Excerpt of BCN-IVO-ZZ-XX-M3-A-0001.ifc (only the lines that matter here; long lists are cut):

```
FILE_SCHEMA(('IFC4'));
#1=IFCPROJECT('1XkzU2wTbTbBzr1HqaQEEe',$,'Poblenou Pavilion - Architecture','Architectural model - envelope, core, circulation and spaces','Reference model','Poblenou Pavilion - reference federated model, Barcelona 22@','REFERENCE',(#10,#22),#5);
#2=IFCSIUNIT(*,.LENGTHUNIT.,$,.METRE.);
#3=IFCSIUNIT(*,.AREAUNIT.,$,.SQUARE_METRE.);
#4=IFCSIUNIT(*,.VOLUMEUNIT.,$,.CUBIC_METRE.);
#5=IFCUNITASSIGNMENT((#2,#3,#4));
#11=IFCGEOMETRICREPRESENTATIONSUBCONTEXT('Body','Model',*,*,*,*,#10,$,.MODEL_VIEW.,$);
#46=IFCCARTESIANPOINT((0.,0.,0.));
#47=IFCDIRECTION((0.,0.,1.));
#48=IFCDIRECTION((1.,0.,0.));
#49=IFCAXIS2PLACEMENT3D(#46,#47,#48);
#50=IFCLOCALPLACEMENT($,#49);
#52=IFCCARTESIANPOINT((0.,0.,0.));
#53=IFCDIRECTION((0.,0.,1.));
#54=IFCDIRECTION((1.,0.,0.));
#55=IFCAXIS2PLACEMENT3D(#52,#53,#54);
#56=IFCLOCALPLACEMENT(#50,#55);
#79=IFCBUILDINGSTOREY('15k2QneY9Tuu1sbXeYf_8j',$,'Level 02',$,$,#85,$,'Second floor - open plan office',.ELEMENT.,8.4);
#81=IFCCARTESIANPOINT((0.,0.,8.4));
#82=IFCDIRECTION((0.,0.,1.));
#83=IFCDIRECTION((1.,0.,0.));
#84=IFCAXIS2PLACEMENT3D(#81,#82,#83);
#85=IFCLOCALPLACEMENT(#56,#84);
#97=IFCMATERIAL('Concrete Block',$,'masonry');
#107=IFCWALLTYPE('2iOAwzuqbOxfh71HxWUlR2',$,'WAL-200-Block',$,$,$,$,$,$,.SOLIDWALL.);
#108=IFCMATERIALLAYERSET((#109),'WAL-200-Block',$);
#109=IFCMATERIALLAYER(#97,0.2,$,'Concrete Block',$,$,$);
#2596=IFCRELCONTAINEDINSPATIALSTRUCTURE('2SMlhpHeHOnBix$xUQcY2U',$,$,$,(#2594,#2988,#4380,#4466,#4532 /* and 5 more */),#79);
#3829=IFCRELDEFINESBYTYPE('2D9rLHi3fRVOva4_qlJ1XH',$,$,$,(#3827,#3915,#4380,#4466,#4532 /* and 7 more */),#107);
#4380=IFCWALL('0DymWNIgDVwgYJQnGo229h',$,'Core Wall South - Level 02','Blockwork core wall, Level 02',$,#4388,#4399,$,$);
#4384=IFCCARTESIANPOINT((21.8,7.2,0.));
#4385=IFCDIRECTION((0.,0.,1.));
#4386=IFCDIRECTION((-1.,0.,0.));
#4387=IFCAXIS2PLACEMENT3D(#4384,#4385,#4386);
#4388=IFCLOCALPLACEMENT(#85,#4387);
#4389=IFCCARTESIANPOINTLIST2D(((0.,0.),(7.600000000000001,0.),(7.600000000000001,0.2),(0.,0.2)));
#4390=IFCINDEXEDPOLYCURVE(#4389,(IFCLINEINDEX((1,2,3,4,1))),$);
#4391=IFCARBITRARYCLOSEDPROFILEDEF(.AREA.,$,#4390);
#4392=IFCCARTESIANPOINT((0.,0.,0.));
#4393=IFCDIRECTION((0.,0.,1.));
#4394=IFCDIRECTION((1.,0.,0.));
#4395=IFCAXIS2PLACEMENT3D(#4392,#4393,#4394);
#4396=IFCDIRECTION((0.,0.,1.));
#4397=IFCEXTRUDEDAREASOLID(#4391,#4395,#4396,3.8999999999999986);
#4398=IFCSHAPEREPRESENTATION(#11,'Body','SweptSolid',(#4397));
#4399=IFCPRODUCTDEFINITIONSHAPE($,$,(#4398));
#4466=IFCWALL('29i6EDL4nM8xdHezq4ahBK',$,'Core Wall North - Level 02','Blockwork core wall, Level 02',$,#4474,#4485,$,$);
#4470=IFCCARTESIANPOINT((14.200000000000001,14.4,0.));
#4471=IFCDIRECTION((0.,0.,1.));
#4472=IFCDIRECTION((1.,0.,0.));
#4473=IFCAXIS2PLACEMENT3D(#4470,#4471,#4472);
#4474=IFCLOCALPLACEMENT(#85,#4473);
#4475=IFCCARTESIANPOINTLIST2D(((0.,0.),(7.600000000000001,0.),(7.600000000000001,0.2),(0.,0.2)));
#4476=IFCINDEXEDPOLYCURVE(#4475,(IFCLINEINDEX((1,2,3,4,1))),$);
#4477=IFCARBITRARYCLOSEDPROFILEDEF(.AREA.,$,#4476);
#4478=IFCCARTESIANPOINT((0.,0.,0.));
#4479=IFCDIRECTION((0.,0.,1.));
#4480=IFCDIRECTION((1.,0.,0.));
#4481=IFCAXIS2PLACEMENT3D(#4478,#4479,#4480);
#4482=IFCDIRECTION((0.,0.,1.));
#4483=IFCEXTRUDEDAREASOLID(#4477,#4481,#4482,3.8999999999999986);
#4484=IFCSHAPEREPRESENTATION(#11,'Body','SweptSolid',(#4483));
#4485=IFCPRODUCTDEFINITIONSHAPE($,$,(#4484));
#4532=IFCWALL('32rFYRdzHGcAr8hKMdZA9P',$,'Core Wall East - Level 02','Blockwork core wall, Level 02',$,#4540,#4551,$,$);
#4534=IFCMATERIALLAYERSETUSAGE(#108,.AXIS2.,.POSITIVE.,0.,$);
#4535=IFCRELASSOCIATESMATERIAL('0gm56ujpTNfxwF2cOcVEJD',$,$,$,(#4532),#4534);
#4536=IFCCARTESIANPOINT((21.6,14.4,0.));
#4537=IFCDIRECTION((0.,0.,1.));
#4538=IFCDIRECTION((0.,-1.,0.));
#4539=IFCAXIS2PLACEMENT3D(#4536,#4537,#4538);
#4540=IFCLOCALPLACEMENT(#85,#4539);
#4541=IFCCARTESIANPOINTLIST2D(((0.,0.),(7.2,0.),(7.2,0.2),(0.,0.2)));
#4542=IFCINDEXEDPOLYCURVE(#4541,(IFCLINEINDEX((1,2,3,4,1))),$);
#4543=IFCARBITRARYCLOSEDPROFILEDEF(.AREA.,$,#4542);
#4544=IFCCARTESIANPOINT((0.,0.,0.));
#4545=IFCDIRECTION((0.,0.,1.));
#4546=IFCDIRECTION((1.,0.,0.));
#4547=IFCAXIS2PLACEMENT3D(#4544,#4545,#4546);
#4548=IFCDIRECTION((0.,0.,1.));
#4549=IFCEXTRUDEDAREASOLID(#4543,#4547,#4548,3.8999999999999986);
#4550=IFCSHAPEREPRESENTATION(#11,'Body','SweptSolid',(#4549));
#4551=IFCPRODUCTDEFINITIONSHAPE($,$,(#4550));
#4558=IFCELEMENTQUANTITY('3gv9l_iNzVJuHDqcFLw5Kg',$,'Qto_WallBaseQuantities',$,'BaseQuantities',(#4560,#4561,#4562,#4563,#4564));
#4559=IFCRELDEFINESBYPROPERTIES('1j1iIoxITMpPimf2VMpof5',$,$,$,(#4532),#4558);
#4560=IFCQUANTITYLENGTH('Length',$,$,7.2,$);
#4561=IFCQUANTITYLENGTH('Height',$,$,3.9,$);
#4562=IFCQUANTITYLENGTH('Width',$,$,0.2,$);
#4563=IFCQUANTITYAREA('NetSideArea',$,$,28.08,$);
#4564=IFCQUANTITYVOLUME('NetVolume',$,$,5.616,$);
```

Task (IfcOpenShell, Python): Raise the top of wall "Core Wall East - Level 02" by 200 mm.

```python
import ifcopenshell
import ifcopenshell.api.pset
import ifcopenshell.geom
import ifcopenshell.util.element
import ifcopenshell.util.representation
import ifcopenshell.util.shape
import ifcopenshell.util.unit

model = ifcopenshell.open("BCN-IVO-ZZ-XX-M3-A-0001.ifc")
area_scale = ifcopenshell.util.unit.calculate_unit_scale(model, "AREAUNIT")
volume_scale = ifcopenshell.util.unit.calculate_unit_scale(model, "VOLUMEUNIT")
settings = ifcopenshell.geom.settings()


def volume(element):
    """Net volume in cubic metres, openings subtracted."""
    shape = ifcopenshell.geom.create_shape(settings, element)
    return ifcopenshell.util.shape.get_volume(shape.geometry)


wall = model.by_guid("32rFYRdzHGcAr8hKMdZA9P")
before = volume(wall)

body = ifcopenshell.util.representation.get_representation(wall, "Model", "Body")
solid = body.Items[0]
old_height = solid.Depth
solid.Depth += 0.2
after = volume(wall)
thickness = 0.2  # wall thickness in metres

# Update the stored height, areas and volumes.
qto = model.by_id(ifcopenshell.util.element.get_pset(wall, "Qto_WallBaseQuantities", should_inherit=False)["id"])
ifcopenshell.api.pset.edit_qto(model, qto=qto, properties={
    "Height": solid.Depth,
    "NetSideArea": after / thickness / area_scale,
    "NetVolume": after / volume_scale,
})

print(f"height {old_height:g} -> {solid.Depth:g}, volume {before:.3f} -> {after:.3f} m3")

model.write("BCN-IVO-ZZ-XX-M3-A-0001_updated.ifc")
```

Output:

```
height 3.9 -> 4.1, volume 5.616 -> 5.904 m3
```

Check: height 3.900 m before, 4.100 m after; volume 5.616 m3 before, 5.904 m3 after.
